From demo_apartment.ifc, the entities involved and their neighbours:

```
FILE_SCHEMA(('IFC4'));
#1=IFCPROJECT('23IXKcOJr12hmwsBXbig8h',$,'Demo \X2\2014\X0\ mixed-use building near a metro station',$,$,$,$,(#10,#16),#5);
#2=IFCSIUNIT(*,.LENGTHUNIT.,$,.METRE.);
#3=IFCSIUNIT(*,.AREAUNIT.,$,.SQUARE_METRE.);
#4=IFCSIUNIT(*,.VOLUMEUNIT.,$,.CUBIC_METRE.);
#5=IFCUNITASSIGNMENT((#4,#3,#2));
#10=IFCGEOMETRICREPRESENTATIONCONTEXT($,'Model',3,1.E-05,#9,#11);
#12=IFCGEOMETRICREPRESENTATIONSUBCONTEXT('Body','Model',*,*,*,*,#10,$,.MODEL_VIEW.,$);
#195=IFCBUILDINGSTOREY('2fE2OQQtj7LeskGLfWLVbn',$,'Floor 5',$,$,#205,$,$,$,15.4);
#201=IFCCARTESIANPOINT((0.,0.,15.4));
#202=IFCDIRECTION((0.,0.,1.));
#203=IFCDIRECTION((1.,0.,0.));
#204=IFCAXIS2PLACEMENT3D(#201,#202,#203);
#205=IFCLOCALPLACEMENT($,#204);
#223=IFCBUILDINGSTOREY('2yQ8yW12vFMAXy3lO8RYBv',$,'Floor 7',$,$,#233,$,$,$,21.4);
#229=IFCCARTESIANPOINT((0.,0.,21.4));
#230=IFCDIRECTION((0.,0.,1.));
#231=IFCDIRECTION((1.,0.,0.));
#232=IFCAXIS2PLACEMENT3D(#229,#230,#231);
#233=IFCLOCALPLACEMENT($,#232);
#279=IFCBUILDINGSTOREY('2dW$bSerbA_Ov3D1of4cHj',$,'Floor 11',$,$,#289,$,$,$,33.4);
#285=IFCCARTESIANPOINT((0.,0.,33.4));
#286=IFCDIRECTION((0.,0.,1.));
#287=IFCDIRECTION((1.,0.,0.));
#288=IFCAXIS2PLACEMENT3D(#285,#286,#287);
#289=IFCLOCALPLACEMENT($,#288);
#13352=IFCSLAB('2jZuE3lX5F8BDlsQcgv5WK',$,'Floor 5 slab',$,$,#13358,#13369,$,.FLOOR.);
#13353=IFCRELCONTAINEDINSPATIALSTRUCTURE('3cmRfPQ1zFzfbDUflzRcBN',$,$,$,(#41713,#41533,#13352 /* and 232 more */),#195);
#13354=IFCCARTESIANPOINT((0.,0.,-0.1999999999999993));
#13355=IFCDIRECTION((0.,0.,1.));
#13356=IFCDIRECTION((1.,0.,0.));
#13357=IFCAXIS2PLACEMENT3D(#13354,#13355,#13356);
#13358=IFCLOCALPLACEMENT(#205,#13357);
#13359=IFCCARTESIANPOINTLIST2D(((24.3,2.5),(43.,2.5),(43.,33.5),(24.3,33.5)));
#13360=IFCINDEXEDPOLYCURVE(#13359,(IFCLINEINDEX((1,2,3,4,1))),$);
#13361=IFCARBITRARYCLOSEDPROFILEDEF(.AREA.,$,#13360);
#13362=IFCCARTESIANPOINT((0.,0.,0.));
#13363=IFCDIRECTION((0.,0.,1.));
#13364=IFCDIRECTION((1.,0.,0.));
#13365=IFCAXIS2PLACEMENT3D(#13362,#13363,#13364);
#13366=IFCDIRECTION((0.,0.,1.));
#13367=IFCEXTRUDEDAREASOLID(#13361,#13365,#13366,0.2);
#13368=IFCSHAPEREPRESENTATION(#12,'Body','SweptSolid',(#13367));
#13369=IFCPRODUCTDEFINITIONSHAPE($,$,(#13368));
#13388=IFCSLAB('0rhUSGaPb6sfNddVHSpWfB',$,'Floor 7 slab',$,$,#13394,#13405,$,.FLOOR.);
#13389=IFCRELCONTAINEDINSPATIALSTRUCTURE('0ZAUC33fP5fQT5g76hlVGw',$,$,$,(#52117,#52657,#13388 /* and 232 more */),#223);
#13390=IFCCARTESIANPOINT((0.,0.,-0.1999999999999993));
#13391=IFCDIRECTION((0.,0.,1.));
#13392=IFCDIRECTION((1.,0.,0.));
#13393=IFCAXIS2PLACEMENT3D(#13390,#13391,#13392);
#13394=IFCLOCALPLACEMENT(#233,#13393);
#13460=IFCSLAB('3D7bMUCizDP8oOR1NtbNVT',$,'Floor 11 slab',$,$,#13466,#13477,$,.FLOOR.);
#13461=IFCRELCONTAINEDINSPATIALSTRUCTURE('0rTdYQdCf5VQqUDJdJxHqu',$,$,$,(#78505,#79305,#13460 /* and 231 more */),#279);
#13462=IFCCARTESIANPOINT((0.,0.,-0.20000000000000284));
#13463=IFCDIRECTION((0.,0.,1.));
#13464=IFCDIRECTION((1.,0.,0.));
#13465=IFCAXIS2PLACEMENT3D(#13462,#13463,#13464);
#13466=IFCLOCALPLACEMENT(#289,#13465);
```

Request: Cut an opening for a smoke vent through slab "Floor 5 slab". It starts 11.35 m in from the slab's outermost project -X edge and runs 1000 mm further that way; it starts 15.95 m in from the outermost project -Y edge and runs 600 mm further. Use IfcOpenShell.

```python
import numpy as np
import ifcopenshell
import ifcopenshell.api.feature
import ifcopenshell.api.geometry
import ifcopenshell.api.root
import ifcopenshell.geom
import ifcopenshell.util.placement
import ifcopenshell.util.representation
import ifcopenshell.util.shape
import ifcopenshell.util.unit

model = ifcopenshell.open("demo_apartment.ifc")
unit_scale = ifcopenshell.util.unit.calculate_unit_scale(model)
settings = ifcopenshell.geom.settings()


def volume(element):
    """Net volume in cubic metres, openings subtracted."""
    shape = ifcopenshell.geom.create_shape(settings, element)
    return ifcopenshell.util.shape.get_volume(shape.geometry)


slab = model.by_guid("2jZuE3lX5F8BDlsQcgv5WK")
before = volume(slab)

# Extent in the slab's own axes, in metres. The edges named are its -X and -Y sides.
slab_shape = ifcopenshell.geom.create_shape(settings, slab)
vertices = ifcopenshell.util.shape.get_vertices(slab_shape.geometry)
x_min, y_min, bottom = vertices.min(axis=0)
top = vertices[:, 2].max()

opening = ifcopenshell.api.root.create_entity(model, ifc_class="IfcOpeningElement", name="Smoke vent opening", predefined_type="OPENING")
context = ifcopenshell.util.representation.get_context(model, "Model", "Body", "MODEL_VIEW")
width, depth = 1, 0.6
outline = [(0.0, 0.0), (width, 0.0), (width, depth), (0.0, depth), (0.0, 0.0)]
# Overshoot both faces by 50 mm so the cut is clean.
shape = ifcopenshell.api.geometry.add_slab_representation(
    model, context=context, depth=top - bottom + 0.1, polyline=outline
)
ifcopenshell.api.geometry.assign_representation(model, product=opening, representation=shape)

matrix = ifcopenshell.util.placement.get_local_placement(slab.ObjectPlacement)
matrix[:, 3] = matrix @ np.append(np.array([x_min + 11.35, y_min + 15.95, bottom - 0.05]) / unit_scale, 1.0)
ifcopenshell.api.geometry.edit_object_placement(model, product=opening, matrix=matrix, is_si=False)
ifcopenshell.api.feature.add_feature(model, feature=opening, element=slab)

after = volume(slab)

print(f"slab volume {before:.3f} -> {after:.3f} m3")

model.write("demo_apartment_rev.ifc")
```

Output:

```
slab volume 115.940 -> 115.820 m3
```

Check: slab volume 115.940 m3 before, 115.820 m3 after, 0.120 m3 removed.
